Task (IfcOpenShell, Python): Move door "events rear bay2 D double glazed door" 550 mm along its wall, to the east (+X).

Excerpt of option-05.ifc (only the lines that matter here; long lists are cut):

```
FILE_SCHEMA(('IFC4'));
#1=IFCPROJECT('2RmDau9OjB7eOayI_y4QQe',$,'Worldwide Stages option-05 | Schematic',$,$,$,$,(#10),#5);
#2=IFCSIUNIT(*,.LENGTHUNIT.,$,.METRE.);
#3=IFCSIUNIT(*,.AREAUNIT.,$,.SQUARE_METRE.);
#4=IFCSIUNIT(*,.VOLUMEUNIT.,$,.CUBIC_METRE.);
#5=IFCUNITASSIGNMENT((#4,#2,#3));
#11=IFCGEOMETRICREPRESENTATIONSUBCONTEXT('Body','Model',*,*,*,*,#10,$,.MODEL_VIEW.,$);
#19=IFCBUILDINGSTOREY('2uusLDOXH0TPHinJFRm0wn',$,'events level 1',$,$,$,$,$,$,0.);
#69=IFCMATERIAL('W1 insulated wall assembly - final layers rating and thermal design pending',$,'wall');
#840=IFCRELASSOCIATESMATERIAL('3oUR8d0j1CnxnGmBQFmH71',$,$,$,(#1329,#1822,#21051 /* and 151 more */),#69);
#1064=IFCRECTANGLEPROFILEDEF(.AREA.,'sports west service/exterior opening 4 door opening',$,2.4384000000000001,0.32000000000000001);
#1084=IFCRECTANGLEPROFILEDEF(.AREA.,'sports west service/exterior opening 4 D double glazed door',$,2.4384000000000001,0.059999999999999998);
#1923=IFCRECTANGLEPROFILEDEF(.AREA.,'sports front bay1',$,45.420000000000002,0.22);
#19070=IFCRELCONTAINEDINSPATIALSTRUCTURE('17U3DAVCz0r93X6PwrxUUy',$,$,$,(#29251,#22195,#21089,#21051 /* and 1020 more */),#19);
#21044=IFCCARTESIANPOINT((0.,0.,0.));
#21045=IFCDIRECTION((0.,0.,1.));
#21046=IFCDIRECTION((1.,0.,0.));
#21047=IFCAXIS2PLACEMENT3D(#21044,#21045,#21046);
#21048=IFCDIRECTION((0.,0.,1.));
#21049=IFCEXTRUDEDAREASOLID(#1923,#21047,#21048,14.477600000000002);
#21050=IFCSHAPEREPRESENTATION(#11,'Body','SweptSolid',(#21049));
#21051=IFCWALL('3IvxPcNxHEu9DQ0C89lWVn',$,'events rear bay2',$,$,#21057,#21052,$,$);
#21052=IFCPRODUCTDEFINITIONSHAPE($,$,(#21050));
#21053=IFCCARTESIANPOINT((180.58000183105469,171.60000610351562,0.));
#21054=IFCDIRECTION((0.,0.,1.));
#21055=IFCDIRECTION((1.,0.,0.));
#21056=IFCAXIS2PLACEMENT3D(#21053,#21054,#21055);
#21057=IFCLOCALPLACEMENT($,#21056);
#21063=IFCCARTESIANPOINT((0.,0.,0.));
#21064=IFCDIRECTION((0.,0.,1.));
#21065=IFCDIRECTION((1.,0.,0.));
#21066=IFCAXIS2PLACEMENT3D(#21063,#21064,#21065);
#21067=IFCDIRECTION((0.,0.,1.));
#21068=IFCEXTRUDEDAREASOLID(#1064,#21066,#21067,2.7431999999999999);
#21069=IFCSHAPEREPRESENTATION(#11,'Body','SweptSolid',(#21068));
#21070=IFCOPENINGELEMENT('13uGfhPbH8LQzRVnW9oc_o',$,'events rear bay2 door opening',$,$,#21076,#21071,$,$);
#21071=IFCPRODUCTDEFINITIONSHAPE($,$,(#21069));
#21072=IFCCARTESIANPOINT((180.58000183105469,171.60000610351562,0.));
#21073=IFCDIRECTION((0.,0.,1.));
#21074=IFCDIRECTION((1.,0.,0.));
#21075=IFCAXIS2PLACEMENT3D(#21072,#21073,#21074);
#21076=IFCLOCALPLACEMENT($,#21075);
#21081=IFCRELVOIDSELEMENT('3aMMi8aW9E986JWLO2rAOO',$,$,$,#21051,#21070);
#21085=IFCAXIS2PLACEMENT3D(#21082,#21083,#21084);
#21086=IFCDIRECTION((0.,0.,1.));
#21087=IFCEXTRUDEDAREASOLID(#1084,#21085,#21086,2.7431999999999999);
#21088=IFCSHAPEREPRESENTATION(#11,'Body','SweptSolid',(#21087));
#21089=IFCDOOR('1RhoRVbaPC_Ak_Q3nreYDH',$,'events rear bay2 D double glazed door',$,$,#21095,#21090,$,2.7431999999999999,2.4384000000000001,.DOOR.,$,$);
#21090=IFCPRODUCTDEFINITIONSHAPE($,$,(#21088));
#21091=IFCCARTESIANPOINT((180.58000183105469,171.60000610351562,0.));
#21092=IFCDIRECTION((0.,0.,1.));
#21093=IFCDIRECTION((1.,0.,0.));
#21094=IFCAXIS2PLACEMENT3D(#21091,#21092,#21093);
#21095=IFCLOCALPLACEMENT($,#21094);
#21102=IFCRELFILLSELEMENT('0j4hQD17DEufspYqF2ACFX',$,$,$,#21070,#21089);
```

```python
import ifcopenshell
import ifcopenshell.api.geometry
import ifcopenshell.util.placement
import ifcopenshell.util.unit

model = ifcopenshell.open("option-05.ifc")
unit_scale = ifcopenshell.util.unit.calculate_unit_scale(model)

door = model.by_id(21089)
opening = door.FillsVoids[0].RelatingOpeningElement
wall = opening.VoidsElements[0].RelatingBuildingElement

wall_matrix = ifcopenshell.util.placement.get_local_placement(wall.ObjectPlacement)
shift = wall_matrix[:3, 0] * 0.55 / unit_scale
before = ifcopenshell.util.placement.get_local_placement(door.ObjectPlacement)[:3, 3].copy()

# The door is not placed relative to its opening, so move both.
for product in (opening, door):
    matrix = ifcopenshell.util.placement.get_local_placement(product.ObjectPlacement)
    matrix[:3, 3] += shift
    ifcopenshell.api.geometry.edit_object_placement(model, product=product, matrix=matrix, is_si=False)

after = ifcopenshell.util.placement.get_local_placement(door.ObjectPlacement)[:3, 3]
print("door moved by", (after - before).round(3) + 0.0)

model.write("option-05_edited.ifc")
```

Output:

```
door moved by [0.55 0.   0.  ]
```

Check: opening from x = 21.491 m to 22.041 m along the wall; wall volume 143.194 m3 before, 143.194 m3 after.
